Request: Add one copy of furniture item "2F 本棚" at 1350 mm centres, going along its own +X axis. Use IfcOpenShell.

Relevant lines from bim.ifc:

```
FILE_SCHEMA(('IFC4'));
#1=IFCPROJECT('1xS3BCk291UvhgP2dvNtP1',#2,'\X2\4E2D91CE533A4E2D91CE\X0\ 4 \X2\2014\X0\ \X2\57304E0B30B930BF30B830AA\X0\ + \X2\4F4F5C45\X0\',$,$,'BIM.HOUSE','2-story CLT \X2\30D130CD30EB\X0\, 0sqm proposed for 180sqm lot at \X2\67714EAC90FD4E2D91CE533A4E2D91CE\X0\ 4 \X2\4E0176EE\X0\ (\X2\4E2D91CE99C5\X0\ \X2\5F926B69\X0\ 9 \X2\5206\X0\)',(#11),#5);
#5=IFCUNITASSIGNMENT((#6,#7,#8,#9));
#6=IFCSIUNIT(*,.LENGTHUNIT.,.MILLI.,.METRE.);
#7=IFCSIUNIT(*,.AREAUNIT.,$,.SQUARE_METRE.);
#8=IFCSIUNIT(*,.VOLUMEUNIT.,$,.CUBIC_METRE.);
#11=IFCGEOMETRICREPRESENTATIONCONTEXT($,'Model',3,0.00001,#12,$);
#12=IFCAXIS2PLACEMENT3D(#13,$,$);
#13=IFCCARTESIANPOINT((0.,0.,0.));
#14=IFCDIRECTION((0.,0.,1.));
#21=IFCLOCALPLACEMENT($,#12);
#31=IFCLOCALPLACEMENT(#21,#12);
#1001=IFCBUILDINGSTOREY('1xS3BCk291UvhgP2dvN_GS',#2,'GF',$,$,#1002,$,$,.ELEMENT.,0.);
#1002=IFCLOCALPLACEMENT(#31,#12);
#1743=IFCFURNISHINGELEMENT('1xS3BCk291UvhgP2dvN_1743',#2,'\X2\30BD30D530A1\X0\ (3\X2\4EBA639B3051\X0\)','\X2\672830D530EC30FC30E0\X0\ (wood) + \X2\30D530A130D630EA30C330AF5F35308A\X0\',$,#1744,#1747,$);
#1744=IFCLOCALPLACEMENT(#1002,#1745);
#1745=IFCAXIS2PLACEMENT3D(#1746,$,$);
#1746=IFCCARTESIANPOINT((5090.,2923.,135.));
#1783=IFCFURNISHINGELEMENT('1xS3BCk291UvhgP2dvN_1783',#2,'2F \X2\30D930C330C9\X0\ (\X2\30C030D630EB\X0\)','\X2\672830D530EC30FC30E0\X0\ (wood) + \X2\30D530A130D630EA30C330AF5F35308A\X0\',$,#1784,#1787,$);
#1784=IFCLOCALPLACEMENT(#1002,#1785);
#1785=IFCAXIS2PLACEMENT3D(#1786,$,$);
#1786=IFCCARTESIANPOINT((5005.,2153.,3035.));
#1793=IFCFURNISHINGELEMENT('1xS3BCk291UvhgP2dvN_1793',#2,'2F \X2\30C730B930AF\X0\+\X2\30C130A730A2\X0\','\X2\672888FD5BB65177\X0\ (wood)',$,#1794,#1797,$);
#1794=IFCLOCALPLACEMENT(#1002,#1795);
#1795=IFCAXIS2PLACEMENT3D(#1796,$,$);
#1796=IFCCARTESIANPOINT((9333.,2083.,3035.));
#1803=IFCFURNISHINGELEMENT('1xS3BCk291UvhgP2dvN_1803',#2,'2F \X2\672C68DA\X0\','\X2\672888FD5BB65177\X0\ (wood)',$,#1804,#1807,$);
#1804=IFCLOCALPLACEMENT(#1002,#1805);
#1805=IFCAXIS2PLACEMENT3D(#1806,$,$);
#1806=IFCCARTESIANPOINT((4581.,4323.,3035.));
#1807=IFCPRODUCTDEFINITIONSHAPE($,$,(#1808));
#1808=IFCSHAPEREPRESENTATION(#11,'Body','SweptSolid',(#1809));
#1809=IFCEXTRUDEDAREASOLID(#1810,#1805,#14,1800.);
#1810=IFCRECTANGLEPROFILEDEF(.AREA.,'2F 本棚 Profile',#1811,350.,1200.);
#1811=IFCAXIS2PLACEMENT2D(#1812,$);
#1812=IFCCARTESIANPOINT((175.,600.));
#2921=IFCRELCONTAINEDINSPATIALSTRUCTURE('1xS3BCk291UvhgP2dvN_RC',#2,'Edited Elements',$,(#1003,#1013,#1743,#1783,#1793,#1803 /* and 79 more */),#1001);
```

```python
import ifcopenshell
import ifcopenshell.api.geometry
import ifcopenshell.api.root
import ifcopenshell.util.element
import ifcopenshell.util.placement

model = ifcopenshell.open("bim.ifc")


def reuse_history(source, copy):
    """copy_class also copies each property set's owner history, people and application; keep the originals."""
    for rel in copy.IsDefinedBy:
        if rel.is_a("IfcRelDefinesByProperties") and (history := rel.RelatingPropertyDefinition.OwnerHistory):
            rel.RelatingPropertyDefinition.OwnerHistory = source.OwnerHistory
            ifcopenshell.util.element.remove_deep2(model, history)


source = model.by_guid("1xS3BCk291UvhgP2dvN_1803")
base = ifcopenshell.util.placement.get_local_placement(source.ObjectPlacement)
step = base[:3, 0] * 1350.0

for i in range(1, 2):
    copy = ifcopenshell.api.root.copy_class(model, product=source)
    copy.Representation = ifcopenshell.util.element.copy_deep(
        model, source.Representation, exclude=["IfcGeometricRepresentationContext", "IfcRepresentationMap"]
    )
    reuse_history(source, copy)
    matrix = base.copy()
    matrix[:3, 3] += i * step
    print("added at", matrix[:3, 3].round(3) + 0.0)
    ifcopenshell.api.geometry.edit_object_placement(model, product=copy, matrix=matrix, is_si=False)

model.write("bim_rev.ifc")
```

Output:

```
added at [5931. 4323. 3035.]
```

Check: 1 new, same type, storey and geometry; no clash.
